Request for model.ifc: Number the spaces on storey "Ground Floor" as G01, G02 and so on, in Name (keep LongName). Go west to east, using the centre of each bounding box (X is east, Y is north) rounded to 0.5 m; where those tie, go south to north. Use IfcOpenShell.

First a look at what the model holds.

```python
import ifcopenshell
import ifcopenshell.util.element
import ifcopenshell.util.placement

model = ifcopenshell.open("model.ifc")
print(model.schema)
storey = next(s for s in model.by_type("IfcBuildingStorey") if s.Name == "Ground Floor")
spaces = [e for e in ifcopenshell.util.element.get_decomposition(storey) if e.is_a("IfcSpace")]
for e in sorted(spaces, key=lambda e: e.id()):
    origin = ifcopenshell.util.placement.get_local_placement(e.ObjectPlacement)[:3, 3]
    print(e.id(), e.Name, e.LongName, origin.round(2) + 0.0, sep=" | ")
```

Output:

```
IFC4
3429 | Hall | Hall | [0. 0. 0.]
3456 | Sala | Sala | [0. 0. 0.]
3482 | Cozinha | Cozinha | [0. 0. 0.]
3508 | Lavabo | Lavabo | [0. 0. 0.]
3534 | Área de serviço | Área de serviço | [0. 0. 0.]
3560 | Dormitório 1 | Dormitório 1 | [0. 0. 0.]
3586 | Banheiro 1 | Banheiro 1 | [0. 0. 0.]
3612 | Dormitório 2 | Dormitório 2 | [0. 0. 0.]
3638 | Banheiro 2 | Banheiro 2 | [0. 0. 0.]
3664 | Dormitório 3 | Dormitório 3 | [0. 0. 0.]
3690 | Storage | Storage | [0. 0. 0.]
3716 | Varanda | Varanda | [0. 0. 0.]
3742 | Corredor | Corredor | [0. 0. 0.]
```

```python
import ifcopenshell
import ifcopenshell.geom
import ifcopenshell.util.element
import ifcopenshell.util.shape

model = ifcopenshell.open("model.ifc")
settings = ifcopenshell.geom.settings()
settings.set("use-world-coords", True)


def centre(element):
    shape = ifcopenshell.geom.create_shape(settings, element)
    return ifcopenshell.util.shape.get_bbox_centroid(shape.geometry)


storey = next(s for s in model.by_type("IfcBuildingStorey") if s.Name == "Ground Floor")
spaces = [e for e in ifcopenshell.util.element.get_decomposition(storey) if e.is_a("IfcSpace")]

# Insertion points can sit at a corner or the storey origin, so sort by the geometry (in metres).
centres = {e: centre(e) for e in spaces}
spaces.sort(key=lambda e: (round(centres[e][0] / 0.5), centres[e][1]))

for i, e in enumerate(spaces, start=1):
    number = f"G{i:02d}"
    e.Name = number
    print(e.id(), number)

model.write("model_updated.ifc")
```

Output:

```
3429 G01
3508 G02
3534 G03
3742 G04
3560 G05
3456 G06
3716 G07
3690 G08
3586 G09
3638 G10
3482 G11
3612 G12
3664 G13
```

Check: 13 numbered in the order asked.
